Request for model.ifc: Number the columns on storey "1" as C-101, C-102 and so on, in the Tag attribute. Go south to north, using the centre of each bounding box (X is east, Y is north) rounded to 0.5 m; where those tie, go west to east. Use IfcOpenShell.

First a look at what the model holds.

```python
import ifcopenshell
import ifcopenshell.util.element
import ifcopenshell.util.placement

model = ifcopenshell.open("model.ifc")
print(model.schema)
storey = next(s for s in model.by_type("IfcBuildingStorey") if s.Name == "1")
columns = [e for e in ifcopenshell.util.element.get_decomposition(storey) if e.is_a("IfcColumn")]
for e in sorted(columns, key=lambda e: e.id()):
    origin = ifcopenshell.util.placement.get_local_placement(e.ObjectPlacement)[:3, 3]
    print(e.id(), e.Tag, e.Name, origin.round(2) + 0.0, sep=" | ")
```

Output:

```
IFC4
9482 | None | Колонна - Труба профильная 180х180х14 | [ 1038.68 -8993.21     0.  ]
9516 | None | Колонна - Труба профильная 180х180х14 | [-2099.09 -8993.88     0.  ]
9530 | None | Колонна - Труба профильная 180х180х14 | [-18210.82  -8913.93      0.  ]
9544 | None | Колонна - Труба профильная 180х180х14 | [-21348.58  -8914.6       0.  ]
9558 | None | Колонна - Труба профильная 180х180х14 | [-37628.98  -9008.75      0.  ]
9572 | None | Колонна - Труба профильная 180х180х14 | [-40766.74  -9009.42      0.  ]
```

```python
import ifcopenshell
import ifcopenshell.geom
import ifcopenshell.util.element
import ifcopenshell.util.shape

model = ifcopenshell.open("model.ifc")
settings = ifcopenshell.geom.settings()
settings.set("use-world-coords", True)


def centre(element):
    shape = ifcopenshell.geom.create_shape(settings, element)
    return ifcopenshell.util.shape.get_bbox_centroid(shape.geometry)


storey = next(s for s in model.by_type("IfcBuildingStorey") if s.Name == "1")
columns = [e for e in ifcopenshell.util.element.get_decomposition(storey) if e.is_a("IfcColumn")]

# Insertion points can sit at a corner or the storey origin, so sort by the geometry (in metres).
centres = {e: centre(e) for e in columns}
columns.sort(key=lambda e: (round(centres[e][1] / 0.5), centres[e][0]))

for i, e in enumerate(columns, start=1):
    number = f"C-1{i:02d}"
    e.Tag = number
    print(e.id(), number)

model.write("model_edited.ifc")
```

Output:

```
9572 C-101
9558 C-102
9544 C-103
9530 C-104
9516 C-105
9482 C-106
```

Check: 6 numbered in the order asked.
